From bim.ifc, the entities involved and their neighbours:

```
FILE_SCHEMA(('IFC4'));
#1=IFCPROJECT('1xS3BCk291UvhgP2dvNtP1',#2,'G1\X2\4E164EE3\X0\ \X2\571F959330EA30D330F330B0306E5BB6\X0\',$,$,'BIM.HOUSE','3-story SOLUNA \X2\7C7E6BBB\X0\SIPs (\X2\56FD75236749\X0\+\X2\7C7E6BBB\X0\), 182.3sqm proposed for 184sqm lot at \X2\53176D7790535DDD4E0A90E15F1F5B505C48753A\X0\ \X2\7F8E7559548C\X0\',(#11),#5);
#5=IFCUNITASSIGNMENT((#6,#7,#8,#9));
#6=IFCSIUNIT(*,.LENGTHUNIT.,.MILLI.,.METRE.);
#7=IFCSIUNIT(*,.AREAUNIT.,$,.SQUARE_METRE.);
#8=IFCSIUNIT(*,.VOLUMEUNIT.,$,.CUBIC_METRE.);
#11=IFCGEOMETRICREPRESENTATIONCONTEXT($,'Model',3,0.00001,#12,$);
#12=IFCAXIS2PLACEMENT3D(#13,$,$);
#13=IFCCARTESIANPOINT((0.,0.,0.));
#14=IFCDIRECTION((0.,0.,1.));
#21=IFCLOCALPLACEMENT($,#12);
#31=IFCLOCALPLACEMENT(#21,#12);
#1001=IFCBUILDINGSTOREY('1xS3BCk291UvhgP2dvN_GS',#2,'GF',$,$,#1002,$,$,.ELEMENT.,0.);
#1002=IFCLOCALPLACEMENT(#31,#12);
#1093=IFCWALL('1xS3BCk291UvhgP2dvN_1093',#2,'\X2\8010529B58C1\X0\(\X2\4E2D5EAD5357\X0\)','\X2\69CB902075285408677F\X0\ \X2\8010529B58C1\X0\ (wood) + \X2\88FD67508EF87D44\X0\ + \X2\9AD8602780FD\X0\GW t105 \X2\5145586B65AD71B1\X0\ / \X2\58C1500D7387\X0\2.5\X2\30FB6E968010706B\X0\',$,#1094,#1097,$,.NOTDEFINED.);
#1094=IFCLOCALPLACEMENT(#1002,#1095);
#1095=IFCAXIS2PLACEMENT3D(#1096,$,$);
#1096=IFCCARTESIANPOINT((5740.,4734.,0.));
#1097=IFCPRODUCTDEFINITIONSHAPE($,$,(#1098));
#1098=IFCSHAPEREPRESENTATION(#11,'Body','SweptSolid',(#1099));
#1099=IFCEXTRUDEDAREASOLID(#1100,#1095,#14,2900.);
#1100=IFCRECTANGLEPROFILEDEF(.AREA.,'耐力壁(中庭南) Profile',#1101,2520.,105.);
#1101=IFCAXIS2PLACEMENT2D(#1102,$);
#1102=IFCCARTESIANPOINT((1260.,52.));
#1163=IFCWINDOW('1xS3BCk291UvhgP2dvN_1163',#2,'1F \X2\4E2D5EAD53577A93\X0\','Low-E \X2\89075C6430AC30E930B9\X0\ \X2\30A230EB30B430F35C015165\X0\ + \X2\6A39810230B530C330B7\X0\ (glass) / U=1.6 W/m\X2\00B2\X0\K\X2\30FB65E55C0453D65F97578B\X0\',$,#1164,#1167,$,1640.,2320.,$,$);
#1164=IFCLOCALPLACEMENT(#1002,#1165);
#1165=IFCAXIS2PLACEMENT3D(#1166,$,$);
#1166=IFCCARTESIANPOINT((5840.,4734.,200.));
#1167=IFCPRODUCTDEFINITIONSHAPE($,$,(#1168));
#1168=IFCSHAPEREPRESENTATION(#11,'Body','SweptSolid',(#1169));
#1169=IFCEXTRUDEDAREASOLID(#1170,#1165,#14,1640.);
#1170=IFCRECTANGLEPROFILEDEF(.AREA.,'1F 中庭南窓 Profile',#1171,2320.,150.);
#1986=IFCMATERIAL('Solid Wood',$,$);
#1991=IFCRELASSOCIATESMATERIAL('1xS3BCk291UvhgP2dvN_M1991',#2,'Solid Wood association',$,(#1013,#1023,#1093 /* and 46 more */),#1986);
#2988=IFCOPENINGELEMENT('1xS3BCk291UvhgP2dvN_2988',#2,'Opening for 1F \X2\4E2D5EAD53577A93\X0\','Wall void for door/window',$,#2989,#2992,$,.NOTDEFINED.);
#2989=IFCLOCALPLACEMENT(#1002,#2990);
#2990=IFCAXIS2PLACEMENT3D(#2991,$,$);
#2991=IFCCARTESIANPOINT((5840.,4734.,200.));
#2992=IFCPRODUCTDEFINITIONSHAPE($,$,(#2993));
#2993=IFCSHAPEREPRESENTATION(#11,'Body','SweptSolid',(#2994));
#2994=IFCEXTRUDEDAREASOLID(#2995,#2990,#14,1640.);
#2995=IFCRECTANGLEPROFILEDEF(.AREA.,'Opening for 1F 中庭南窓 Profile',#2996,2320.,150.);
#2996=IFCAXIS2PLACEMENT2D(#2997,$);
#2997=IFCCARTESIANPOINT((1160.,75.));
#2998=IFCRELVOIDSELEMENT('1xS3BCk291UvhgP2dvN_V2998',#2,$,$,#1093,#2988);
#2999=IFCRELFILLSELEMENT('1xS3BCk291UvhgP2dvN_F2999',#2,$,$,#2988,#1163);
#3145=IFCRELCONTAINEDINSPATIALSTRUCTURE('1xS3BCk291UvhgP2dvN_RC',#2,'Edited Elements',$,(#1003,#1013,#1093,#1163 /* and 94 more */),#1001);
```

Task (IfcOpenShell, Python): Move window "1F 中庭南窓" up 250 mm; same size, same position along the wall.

```python
import numpy as np
import ifcopenshell
import ifcopenshell.api.geometry
import ifcopenshell.util.placement
import ifcopenshell.util.unit

model = ifcopenshell.open("bim.ifc")
unit_scale = ifcopenshell.util.unit.calculate_unit_scale(model)

window = model.by_guid("1xS3BCk291UvhgP2dvN_1163")
opening = window.FillsVoids[0].RelatingOpeningElement
dz = 250.0

shift = np.array([0.0, 0.0, dz])
# The window is not placed relative to its opening, so move both.
for product in (opening, window):
    matrix = ifcopenshell.util.placement.get_local_placement(product.ObjectPlacement)
    matrix[:3, 3] += shift
    ifcopenshell.api.geometry.edit_object_placement(model, product=product, matrix=matrix, is_si=False)

print(f"moved by {dz * unit_scale:+.3f} m")

model.write("bim_rev.ifc")
```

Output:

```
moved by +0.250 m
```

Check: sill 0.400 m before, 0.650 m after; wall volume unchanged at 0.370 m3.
